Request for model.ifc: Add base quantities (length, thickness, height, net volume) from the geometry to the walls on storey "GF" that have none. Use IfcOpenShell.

First a look at what the model holds.

```python
import ifcopenshell
import ifcopenshell.util.element
import ifcopenshell.util.unit

model = ifcopenshell.open("model.ifc")
print(model.schema)
for unit_type in ("LENGTHUNIT", "AREAUNIT", "VOLUMEUNIT"):
    print(unit_type, ifcopenshell.util.unit.calculate_unit_scale(model, unit_type))
storey = next(s for s in model.by_type("IfcBuildingStorey") if s.Name == "GF")
walls = [e for e in ifcopenshell.util.element.get_decomposition(storey) if e.is_a("IfcWall")]
for e in sorted(walls, key=lambda e: e.id()):
    print(e.id(), e.is_a(), e.Name, list(ifcopenshell.util.element.get_psets(e, qtos_only=True)), sep=" | ")
```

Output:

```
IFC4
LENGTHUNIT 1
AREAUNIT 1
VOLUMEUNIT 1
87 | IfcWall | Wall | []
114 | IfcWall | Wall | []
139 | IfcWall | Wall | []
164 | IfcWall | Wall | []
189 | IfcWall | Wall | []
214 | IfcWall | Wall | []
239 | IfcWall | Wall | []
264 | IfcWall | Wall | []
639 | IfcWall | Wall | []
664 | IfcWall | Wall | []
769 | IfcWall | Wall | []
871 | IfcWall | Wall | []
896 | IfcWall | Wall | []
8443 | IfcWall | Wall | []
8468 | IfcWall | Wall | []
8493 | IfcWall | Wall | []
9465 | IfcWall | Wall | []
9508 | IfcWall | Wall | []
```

```python
import ifcopenshell
import ifcopenshell.api.pset
import ifcopenshell.geom
import ifcopenshell.util.element
import ifcopenshell.util.shape
import ifcopenshell.util.unit

model = ifcopenshell.open("model.ifc")
unit_scale = ifcopenshell.util.unit.calculate_unit_scale(model)
volume_scale = ifcopenshell.util.unit.calculate_unit_scale(model, "VOLUMEUNIT")
settings = ifcopenshell.geom.settings()

storey = next(s for s in model.by_type("IfcBuildingStorey") if s.Name == "GF")
walls = [e for e in ifcopenshell.util.element.get_decomposition(storey) if e.is_a("IfcWall")]

for e in sorted(walls, key=lambda e: e.id()):
    if ifcopenshell.util.element.get_psets(e, qtos_only=True, should_inherit=False):
        continue
    # Geometry comes back in metres, in the element's own axes.
    shape = ifcopenshell.geom.create_shape(settings, e)
    values = {
        "Length": ifcopenshell.util.shape.get_x(shape.geometry) / unit_scale,
        "Width": ifcopenshell.util.shape.get_y(shape.geometry) / unit_scale,
        "Height": ifcopenshell.util.shape.get_z(shape.geometry) / unit_scale,
        "NetVolume": ifcopenshell.util.shape.get_volume(shape.geometry) / volume_scale,
    }
    qto = ifcopenshell.api.pset.add_qto(model, product=e, name="Qto_WallBaseQuantities")
    ifcopenshell.api.pset.edit_qto(model, qto=qto, properties=values)
    print(e.id(), {k: round(v, 3) for k, v in values.items()})

model.write("model_updated.ifc")
```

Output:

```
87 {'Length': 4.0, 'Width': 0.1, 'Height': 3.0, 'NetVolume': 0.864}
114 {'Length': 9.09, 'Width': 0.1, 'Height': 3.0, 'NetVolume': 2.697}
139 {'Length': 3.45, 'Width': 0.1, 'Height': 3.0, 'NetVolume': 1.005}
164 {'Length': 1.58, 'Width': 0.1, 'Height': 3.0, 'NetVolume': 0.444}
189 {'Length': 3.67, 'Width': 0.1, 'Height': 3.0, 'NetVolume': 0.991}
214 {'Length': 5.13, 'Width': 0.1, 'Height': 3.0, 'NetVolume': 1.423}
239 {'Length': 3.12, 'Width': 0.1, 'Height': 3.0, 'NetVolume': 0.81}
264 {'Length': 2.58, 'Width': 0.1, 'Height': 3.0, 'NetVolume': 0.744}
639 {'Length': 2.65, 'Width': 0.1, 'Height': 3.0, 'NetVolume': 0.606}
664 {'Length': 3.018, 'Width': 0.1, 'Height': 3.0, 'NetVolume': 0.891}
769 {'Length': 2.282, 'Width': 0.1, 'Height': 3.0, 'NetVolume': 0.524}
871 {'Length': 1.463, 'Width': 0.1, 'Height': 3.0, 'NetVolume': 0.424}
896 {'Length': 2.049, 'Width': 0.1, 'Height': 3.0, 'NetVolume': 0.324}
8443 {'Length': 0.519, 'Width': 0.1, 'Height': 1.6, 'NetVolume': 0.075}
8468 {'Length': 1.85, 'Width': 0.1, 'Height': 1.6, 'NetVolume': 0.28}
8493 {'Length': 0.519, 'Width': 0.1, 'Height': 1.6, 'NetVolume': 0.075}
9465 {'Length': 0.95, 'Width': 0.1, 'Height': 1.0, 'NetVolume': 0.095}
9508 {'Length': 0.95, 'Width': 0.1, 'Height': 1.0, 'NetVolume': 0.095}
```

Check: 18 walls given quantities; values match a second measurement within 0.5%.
